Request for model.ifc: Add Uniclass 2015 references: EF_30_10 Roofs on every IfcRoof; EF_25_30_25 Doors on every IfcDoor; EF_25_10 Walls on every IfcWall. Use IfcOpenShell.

First a look at what the model holds.

```python
import ifcopenshell

model = ifcopenshell.open("model.ifc")
print(model.schema)
print("classifications:", [c.Name for c in model.by_type("IfcClassification")])
for ifc_class in ("IfcDoor", "IfcRoof", "IfcStair", "IfcWall", "IfcWindow"):
    print(ifc_class, len(model.by_type(ifc_class)))
```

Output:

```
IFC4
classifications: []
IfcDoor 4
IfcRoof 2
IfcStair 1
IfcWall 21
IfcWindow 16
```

```python
import ifcopenshell
import ifcopenshell.api.classification

model = ifcopenshell.open("model.ifc")

system = ifcopenshell.api.classification.add_classification(model, classification="Uniclass 2015")

codes = {
    "IfcRoof": ("EF_30_10", "Roofs"),
    "IfcDoor": ("EF_25_30_25", "Doors"),
    "IfcWall": ("EF_25_10", "Walls"),
}
for ifc_class, (code, name) in codes.items():
    products = model.by_type(ifc_class)
    ifcopenshell.api.classification.add_reference(
        model, products=products, classification=system, identification=code, name=name
    )
    print(code, len(products))

model.write("model_rev.ifc")
```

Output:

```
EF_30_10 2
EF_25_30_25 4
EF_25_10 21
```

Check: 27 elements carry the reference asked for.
